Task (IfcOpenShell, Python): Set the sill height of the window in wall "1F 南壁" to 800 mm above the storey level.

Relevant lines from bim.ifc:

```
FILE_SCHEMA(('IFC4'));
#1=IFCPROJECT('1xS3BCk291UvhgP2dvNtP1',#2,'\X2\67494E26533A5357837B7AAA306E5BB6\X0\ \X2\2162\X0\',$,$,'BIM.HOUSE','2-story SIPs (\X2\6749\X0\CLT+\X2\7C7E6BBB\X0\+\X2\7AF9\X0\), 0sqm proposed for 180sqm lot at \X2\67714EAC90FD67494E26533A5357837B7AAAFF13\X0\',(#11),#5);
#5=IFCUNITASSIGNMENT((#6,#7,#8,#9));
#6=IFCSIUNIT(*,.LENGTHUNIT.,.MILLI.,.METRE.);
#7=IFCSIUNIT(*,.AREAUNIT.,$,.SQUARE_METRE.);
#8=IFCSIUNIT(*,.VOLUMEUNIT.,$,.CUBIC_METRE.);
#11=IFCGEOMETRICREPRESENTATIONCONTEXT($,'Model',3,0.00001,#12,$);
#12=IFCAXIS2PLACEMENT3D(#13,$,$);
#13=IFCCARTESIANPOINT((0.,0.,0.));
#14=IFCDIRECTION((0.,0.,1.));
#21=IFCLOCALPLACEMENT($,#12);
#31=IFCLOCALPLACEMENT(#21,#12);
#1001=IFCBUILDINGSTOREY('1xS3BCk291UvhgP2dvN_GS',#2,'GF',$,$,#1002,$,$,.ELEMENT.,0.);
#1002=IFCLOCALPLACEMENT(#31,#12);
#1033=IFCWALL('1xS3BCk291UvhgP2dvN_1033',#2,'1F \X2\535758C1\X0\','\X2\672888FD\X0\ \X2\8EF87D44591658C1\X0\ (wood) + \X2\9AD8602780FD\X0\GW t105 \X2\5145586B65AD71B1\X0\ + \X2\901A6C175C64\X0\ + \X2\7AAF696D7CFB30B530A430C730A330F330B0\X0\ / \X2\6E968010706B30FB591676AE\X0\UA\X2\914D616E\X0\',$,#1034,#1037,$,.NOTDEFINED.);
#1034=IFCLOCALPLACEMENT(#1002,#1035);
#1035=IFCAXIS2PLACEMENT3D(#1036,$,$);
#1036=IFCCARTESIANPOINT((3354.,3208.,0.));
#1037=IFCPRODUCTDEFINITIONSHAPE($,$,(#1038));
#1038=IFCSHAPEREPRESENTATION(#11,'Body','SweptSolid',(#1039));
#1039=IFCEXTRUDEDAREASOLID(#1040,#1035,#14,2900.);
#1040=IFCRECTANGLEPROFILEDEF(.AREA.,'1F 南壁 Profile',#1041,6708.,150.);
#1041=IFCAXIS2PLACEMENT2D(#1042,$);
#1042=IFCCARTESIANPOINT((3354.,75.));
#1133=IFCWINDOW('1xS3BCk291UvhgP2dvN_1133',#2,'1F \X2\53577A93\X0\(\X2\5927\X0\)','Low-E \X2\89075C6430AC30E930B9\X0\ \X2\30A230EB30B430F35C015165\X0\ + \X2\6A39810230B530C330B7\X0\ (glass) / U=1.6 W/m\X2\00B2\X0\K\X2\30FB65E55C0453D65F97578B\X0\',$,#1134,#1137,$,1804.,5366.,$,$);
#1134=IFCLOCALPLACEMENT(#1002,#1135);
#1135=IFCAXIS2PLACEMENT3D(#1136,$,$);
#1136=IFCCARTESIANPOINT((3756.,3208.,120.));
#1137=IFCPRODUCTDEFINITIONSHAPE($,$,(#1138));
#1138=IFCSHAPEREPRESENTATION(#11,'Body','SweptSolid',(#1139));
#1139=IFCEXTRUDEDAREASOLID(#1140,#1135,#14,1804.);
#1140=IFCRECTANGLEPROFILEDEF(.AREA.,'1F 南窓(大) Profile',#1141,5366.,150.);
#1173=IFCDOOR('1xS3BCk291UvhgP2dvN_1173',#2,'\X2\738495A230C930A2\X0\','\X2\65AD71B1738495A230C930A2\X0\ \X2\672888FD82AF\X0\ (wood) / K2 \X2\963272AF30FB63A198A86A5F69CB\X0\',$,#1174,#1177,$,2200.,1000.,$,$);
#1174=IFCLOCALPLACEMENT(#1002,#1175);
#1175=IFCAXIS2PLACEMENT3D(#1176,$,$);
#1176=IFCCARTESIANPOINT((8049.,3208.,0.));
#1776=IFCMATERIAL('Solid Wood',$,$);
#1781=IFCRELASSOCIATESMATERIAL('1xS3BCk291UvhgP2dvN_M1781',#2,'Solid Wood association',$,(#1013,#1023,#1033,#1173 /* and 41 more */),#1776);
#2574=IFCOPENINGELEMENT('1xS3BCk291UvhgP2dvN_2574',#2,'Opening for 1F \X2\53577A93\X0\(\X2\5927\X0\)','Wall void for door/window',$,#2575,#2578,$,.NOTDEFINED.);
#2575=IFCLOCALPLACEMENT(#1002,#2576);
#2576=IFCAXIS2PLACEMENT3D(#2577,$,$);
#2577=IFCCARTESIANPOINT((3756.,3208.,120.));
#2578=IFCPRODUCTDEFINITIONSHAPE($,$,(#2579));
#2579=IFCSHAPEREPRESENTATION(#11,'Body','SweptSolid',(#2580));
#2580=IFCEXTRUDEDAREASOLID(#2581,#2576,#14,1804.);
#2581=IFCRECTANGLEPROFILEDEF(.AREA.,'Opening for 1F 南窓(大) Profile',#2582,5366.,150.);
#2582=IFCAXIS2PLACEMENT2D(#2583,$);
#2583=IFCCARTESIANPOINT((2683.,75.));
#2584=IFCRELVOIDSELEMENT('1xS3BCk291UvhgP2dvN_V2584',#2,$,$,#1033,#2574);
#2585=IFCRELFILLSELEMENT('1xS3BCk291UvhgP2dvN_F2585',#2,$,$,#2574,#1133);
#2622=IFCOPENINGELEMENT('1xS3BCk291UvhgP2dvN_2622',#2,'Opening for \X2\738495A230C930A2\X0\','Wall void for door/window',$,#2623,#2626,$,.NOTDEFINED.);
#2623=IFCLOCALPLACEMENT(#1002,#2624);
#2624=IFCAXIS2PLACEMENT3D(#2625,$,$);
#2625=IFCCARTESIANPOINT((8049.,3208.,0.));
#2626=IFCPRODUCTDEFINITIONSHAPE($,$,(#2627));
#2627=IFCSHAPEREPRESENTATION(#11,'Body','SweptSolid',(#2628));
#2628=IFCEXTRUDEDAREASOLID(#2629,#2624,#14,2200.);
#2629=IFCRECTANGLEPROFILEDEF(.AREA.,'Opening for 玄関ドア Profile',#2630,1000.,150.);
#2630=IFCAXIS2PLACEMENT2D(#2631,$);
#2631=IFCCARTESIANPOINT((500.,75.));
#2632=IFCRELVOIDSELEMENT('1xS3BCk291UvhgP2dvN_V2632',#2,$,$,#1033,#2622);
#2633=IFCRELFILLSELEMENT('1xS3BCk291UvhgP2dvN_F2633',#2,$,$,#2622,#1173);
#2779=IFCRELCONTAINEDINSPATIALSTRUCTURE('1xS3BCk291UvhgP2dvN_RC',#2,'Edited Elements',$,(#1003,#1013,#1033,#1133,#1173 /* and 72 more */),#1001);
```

```python
import numpy as np
import ifcopenshell
import ifcopenshell.api.geometry
import ifcopenshell.geom
import ifcopenshell.util.element
import ifcopenshell.util.placement
import ifcopenshell.util.shape
import ifcopenshell.util.unit

model = ifcopenshell.open("bim.ifc")
unit_scale = ifcopenshell.util.unit.calculate_unit_scale(model)

window = model.by_guid("1xS3BCk291UvhgP2dvN_1133")
opening = window.FillsVoids[0].RelatingOpeningElement
storey = ifcopenshell.util.element.get_container(window, ifc_class="IfcBuildingStorey")
level = ifcopenshell.util.placement.get_local_placement(storey.ObjectPlacement)[2, 3]

# The opening's origin need not be at the sill, so measure its lowest point.
shape = ifcopenshell.geom.create_shape(ifcopenshell.geom.settings(), opening)
bottom = ifcopenshell.util.shape.get_shape_bottom_elevation(shape, shape.geometry) / unit_scale
dz = level + 0.8 / unit_scale - bottom

shift = np.array([0.0, 0.0, dz])
# The window is not placed relative to its opening, so move both.
for product in (opening, window):
    matrix = ifcopenshell.util.placement.get_local_placement(product.ObjectPlacement)
    matrix[:3, 3] += shift
    ifcopenshell.api.geometry.edit_object_placement(model, product=product, matrix=matrix, is_si=False)

print(f"moved by {dz * unit_scale:+.3f} m")

model.write("bim_updated.ifc")
```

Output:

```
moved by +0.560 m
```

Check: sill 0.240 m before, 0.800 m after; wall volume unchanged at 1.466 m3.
